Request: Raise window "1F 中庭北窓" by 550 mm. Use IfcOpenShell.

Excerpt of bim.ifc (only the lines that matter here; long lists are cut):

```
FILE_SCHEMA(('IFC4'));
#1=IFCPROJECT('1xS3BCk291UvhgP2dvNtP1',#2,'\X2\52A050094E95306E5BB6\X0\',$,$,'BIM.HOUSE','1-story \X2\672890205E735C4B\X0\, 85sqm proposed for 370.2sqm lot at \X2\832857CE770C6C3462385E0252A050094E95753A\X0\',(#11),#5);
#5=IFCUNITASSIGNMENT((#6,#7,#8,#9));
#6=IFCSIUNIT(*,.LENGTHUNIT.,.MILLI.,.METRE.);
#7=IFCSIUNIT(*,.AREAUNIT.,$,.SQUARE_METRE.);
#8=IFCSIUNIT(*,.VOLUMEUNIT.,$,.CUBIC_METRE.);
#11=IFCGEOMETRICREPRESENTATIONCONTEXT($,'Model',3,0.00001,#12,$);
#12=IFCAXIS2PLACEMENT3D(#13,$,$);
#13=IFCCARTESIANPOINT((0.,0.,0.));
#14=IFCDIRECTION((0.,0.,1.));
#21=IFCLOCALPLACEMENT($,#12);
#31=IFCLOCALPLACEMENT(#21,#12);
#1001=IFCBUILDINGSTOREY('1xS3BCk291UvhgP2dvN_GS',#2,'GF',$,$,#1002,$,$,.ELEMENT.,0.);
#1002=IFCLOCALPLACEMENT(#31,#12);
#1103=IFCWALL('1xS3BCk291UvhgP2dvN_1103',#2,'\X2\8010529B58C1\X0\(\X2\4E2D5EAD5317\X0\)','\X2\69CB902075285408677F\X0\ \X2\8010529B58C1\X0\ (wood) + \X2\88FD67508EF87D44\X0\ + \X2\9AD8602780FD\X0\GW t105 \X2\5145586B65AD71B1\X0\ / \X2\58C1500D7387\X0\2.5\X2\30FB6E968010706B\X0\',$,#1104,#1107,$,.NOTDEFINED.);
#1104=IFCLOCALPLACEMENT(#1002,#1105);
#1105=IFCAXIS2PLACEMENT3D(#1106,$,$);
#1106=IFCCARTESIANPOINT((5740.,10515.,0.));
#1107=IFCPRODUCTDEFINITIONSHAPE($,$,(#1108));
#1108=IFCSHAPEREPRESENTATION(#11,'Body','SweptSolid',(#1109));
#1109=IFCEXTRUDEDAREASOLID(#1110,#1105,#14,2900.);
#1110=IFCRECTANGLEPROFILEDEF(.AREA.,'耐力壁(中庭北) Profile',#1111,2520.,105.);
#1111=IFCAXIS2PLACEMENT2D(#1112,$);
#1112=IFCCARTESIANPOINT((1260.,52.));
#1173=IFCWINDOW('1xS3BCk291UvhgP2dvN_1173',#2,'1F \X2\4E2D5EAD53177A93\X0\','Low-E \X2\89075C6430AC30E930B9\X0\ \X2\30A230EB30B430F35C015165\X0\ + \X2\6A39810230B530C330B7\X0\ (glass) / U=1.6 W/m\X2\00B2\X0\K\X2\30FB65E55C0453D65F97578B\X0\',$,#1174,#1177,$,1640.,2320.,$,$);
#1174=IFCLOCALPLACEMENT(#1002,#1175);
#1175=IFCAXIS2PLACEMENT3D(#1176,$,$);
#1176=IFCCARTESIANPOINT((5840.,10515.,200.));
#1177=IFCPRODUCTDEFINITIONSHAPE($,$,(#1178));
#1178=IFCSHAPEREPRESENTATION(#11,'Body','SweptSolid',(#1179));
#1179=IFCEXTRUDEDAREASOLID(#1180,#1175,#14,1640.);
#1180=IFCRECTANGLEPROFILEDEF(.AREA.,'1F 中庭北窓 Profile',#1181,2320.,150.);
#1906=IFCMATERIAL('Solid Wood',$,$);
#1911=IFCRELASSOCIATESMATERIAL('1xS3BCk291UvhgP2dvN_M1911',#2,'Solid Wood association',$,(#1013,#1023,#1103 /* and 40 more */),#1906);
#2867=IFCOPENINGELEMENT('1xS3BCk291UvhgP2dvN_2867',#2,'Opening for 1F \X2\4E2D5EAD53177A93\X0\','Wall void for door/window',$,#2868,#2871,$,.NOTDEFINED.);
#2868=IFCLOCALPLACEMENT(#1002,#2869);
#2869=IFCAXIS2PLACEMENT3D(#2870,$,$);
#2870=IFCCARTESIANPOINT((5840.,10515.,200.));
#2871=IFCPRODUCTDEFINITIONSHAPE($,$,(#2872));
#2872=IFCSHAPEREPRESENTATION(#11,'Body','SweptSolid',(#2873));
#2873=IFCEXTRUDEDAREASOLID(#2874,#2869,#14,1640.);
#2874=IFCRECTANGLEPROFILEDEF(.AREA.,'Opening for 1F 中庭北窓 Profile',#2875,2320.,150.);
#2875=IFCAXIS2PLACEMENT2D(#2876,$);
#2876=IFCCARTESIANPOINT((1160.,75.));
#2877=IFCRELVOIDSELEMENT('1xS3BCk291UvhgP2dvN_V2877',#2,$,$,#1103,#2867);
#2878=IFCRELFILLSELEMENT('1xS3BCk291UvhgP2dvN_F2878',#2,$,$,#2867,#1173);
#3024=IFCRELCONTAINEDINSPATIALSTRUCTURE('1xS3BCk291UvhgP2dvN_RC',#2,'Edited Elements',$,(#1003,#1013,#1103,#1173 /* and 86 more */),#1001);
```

```python
import numpy as np
import ifcopenshell
import ifcopenshell.api.geometry
import ifcopenshell.util.placement
import ifcopenshell.util.unit

model = ifcopenshell.open("bim.ifc")
unit_scale = ifcopenshell.util.unit.calculate_unit_scale(model)

window = model.by_id(1173)
opening = window.FillsVoids[0].RelatingOpeningElement
dz = 0.55 / unit_scale

shift = np.array([0.0, 0.0, dz])
# The window is not placed relative to its opening, so move both.
for product in (opening, window):
    matrix = ifcopenshell.util.placement.get_local_placement(product.ObjectPlacement)
    matrix[:3, 3] += shift
    ifcopenshell.api.geometry.edit_object_placement(model, product=product, matrix=matrix, is_si=False)

print(f"moved by {dz * unit_scale:+.3f} m")

model.write("bim_rev.ifc")
```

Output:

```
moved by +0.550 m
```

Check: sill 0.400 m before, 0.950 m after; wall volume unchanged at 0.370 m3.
